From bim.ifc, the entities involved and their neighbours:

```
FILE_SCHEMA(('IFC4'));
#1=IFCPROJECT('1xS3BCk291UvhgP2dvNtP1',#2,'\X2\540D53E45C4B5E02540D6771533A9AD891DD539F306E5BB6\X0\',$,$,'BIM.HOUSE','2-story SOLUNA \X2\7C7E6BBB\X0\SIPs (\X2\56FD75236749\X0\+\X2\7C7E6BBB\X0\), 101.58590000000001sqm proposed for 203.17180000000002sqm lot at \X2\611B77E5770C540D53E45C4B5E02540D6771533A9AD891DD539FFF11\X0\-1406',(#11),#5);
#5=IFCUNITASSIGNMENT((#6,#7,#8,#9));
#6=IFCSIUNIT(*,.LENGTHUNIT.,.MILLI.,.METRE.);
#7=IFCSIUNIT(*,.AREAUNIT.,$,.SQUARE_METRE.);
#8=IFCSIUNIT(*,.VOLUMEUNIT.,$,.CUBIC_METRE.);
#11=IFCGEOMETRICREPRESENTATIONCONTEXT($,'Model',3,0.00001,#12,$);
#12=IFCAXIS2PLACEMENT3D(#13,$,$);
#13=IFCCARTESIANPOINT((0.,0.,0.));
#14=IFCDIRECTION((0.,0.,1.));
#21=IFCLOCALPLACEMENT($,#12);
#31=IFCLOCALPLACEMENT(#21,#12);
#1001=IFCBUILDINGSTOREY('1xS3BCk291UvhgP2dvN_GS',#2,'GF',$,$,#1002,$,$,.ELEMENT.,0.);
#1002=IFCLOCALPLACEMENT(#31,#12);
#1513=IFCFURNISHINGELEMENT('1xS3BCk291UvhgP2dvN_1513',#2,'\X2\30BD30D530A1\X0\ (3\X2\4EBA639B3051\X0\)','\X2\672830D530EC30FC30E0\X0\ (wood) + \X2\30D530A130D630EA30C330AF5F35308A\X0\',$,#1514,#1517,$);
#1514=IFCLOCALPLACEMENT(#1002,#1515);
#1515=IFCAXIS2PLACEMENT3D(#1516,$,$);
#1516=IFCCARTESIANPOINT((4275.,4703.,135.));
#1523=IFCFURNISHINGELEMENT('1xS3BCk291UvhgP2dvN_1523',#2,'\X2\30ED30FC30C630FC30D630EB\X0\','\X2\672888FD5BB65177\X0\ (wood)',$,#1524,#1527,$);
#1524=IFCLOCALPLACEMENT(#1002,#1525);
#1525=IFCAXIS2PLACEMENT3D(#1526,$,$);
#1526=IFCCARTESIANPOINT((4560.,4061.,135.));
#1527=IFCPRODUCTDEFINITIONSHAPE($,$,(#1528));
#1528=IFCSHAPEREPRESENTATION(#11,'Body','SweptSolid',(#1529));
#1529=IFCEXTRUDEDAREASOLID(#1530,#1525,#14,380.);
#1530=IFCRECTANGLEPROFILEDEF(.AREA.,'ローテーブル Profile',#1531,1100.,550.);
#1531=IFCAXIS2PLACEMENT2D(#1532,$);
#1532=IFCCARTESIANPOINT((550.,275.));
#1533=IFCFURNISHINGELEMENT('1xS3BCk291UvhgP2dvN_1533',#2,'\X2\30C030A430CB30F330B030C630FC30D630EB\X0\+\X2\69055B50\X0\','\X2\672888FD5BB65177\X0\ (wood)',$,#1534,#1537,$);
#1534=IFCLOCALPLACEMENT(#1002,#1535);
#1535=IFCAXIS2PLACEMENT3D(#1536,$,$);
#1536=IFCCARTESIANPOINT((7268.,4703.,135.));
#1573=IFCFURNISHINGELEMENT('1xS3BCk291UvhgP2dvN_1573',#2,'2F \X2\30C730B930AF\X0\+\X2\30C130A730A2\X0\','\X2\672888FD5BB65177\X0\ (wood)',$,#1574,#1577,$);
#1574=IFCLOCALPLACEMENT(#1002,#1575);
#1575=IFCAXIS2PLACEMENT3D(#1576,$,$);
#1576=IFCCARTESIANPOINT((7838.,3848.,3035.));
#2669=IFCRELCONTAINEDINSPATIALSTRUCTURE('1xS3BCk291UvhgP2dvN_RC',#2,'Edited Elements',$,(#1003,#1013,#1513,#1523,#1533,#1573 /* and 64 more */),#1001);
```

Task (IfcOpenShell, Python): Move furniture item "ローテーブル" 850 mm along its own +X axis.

```python
import ifcopenshell
import ifcopenshell.api.geometry
import ifcopenshell.util.placement

model = ifcopenshell.open("bim.ifc")

item = model.by_guid("1xS3BCk291UvhgP2dvN_1523")
matrix = ifcopenshell.util.placement.get_local_placement(item.ObjectPlacement)
matrix[:3, 3] += matrix[:3, 0] * 850.0
ifcopenshell.api.geometry.edit_object_placement(model, product=item, matrix=matrix, is_si=False)

print(ifcopenshell.util.placement.get_local_placement(item.ObjectPlacement).round(3) + 0.0)

model.write("bim_updated.ifc")
```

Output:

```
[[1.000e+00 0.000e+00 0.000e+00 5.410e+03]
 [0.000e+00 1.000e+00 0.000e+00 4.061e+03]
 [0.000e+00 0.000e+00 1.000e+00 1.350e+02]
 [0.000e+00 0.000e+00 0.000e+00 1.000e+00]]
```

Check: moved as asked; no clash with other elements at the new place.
